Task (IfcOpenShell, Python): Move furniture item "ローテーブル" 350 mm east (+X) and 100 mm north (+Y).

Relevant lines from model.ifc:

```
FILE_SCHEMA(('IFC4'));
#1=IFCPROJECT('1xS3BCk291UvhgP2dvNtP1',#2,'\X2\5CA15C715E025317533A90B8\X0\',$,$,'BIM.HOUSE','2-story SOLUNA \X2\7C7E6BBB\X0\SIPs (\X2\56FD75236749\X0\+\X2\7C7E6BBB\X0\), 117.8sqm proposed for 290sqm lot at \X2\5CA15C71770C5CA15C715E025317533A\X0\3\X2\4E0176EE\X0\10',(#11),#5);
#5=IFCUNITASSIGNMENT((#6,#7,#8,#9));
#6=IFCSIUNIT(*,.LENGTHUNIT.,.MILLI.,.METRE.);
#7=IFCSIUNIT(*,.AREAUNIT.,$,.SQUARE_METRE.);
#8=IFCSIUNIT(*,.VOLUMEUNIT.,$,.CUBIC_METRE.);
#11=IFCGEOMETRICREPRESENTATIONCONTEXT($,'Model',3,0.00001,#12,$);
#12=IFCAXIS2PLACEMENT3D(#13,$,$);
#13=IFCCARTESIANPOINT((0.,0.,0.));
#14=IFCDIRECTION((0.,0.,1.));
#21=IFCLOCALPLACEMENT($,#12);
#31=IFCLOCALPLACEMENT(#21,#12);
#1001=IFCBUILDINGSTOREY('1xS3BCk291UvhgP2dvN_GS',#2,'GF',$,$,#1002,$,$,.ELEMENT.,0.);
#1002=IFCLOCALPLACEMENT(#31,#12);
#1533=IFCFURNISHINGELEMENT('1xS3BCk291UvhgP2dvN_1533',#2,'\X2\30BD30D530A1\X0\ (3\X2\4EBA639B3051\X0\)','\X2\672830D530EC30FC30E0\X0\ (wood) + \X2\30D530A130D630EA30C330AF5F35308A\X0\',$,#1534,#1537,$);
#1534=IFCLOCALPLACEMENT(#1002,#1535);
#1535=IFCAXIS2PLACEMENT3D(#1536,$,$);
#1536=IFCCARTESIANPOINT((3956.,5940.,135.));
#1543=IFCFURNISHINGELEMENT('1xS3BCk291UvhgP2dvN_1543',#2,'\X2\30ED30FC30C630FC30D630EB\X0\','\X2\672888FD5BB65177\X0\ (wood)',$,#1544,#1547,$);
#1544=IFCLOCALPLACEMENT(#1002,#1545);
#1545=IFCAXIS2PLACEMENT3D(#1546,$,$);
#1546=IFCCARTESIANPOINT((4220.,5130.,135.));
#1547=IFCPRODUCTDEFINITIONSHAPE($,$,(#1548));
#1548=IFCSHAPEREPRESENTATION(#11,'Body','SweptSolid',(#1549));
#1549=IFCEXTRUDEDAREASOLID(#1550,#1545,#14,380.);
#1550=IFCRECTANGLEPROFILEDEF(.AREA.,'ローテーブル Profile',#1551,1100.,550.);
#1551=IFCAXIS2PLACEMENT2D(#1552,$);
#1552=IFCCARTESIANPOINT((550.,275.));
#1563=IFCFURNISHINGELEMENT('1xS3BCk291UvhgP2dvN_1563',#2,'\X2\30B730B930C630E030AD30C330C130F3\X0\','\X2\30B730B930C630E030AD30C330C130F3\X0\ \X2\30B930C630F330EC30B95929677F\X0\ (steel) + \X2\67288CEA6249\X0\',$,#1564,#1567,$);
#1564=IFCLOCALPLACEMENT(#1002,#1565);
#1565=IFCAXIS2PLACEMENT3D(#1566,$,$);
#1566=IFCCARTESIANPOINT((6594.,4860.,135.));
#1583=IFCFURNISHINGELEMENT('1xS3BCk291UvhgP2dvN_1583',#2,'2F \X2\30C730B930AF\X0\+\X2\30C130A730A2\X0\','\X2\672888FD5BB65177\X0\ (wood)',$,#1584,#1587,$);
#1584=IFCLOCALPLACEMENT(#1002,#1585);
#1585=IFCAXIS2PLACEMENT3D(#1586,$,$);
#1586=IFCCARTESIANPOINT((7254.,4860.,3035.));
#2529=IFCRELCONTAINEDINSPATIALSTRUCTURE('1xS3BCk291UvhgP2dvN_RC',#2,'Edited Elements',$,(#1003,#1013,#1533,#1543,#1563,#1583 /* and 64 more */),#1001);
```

```python
import ifcopenshell
import ifcopenshell.api.geometry
import ifcopenshell.util.placement
import ifcopenshell.util.unit

model = ifcopenshell.open("model.ifc")
unit_scale = ifcopenshell.util.unit.calculate_unit_scale(model)

item = model.by_guid("1xS3BCk291UvhgP2dvN_1543")
matrix = ifcopenshell.util.placement.get_local_placement(item.ObjectPlacement)
matrix[0, 3] += 0.35 / unit_scale
matrix[1, 3] += 0.1 / unit_scale
ifcopenshell.api.geometry.edit_object_placement(model, product=item, matrix=matrix, is_si=False)

print(ifcopenshell.util.placement.get_local_placement(item.ObjectPlacement).round(3) + 0.0)

model.write("model_rev.ifc")
```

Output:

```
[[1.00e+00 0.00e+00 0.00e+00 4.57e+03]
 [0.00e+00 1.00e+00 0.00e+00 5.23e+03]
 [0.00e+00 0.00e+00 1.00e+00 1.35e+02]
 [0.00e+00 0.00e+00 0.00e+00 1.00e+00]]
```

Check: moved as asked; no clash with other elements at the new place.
